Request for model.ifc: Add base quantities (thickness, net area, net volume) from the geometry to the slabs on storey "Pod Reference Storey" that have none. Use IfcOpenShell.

First a look at what the model holds.

```python
import ifcopenshell
import ifcopenshell.util.element
import ifcopenshell.util.unit

model = ifcopenshell.open("model.ifc")
print(model.schema)
for unit_type in ("LENGTHUNIT", "AREAUNIT", "VOLUMEUNIT"):
    print(unit_type, ifcopenshell.util.unit.calculate_unit_scale(model, unit_type))
storey = next(s for s in model.by_type("IfcBuildingStorey") if s.Name == "Pod Reference Storey")
slabs = [e for e in ifcopenshell.util.element.get_decomposition(storey) if e.is_a("IfcSlab")]
for e in sorted(slabs, key=lambda e: e.id()):
    print(e.id(), e.is_a(), e.Name, list(ifcopenshell.util.element.get_psets(e, qtos_only=True)), sep=" | ")
```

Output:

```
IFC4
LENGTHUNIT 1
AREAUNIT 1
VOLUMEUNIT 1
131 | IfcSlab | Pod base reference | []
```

```python
import ifcopenshell
import ifcopenshell.api.pset
import ifcopenshell.geom
import ifcopenshell.util.element
import ifcopenshell.util.shape
import ifcopenshell.util.unit

model = ifcopenshell.open("model.ifc")
unit_scale = ifcopenshell.util.unit.calculate_unit_scale(model)
area_scale = ifcopenshell.util.unit.calculate_unit_scale(model, "AREAUNIT")
volume_scale = ifcopenshell.util.unit.calculate_unit_scale(model, "VOLUMEUNIT")
settings = ifcopenshell.geom.settings()

storey = next(s for s in model.by_type("IfcBuildingStorey") if s.Name == "Pod Reference Storey")
slabs = [e for e in ifcopenshell.util.element.get_decomposition(storey) if e.is_a("IfcSlab")]

for e in sorted(slabs, key=lambda e: e.id()):
    if ifcopenshell.util.element.get_psets(e, qtos_only=True, should_inherit=False):
        continue
    # Geometry comes back in metres, in the element's own axes.
    shape = ifcopenshell.geom.create_shape(settings, e)
    values = {
        "Width": ifcopenshell.util.shape.get_z(shape.geometry) / unit_scale,
        "NetArea": ifcopenshell.util.shape.get_footprint_area(shape.geometry) / area_scale,
        "NetVolume": ifcopenshell.util.shape.get_volume(shape.geometry) / volume_scale,
    }
    qto = ifcopenshell.api.pset.add_qto(model, product=e, name="Qto_SlabBaseQuantities")
    ifcopenshell.api.pset.edit_qto(model, qto=qto, properties=values)
    print(e.id(), {k: round(v, 3) for k, v in values.items()})

model.write("model_updated.ifc")
```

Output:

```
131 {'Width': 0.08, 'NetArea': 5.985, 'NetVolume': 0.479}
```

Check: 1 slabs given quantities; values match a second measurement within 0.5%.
